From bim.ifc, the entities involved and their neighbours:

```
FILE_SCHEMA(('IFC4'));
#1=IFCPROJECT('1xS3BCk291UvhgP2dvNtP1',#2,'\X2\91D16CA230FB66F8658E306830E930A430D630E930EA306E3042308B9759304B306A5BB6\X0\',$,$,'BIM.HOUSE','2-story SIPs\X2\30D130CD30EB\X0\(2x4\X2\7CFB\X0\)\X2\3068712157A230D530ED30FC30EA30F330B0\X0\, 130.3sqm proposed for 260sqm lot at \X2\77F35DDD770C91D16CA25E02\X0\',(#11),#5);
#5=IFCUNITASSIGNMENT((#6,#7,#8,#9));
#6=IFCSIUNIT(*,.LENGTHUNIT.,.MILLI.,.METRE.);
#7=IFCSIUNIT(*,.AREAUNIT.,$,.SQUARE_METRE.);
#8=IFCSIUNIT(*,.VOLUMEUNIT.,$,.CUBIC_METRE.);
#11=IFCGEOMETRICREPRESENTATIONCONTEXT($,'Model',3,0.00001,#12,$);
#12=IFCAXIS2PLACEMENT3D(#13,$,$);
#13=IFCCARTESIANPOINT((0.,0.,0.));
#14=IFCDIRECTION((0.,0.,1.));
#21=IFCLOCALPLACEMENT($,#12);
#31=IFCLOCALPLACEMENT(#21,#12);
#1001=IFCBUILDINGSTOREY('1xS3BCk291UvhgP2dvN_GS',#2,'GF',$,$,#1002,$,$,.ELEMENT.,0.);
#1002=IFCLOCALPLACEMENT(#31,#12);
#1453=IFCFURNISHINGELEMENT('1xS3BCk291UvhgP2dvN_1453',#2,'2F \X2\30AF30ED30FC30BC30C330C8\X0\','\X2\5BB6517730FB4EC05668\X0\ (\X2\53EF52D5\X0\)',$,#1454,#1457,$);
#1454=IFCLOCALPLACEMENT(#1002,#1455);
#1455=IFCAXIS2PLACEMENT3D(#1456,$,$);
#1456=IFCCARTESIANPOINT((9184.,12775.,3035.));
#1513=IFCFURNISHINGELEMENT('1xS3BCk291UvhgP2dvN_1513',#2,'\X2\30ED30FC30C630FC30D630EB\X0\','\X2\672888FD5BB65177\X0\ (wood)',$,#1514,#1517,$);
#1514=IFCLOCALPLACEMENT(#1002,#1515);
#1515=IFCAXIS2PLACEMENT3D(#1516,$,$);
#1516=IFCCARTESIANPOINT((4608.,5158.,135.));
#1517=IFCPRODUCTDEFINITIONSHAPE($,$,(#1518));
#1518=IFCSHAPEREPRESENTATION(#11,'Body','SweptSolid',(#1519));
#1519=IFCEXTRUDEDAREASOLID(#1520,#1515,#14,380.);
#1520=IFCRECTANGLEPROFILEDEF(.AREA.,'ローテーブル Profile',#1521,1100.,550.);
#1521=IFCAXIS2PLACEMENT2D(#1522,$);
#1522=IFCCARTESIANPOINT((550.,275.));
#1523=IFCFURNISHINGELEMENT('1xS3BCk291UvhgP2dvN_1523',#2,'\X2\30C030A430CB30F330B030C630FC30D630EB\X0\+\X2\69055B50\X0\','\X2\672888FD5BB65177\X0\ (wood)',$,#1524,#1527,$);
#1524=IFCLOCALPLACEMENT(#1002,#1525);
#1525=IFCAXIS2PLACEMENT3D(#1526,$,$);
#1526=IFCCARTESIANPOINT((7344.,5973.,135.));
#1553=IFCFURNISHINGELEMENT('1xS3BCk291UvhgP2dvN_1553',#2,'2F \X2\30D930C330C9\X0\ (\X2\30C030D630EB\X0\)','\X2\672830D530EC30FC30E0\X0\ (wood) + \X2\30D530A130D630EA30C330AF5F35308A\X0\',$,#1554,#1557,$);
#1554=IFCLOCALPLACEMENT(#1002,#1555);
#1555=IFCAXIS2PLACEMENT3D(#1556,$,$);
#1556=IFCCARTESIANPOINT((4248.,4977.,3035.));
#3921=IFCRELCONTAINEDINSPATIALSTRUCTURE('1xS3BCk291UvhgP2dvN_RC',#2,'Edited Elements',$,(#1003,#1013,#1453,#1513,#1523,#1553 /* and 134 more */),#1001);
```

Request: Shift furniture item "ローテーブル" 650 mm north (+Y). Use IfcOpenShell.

```python
import ifcopenshell
import ifcopenshell.api.geometry
import ifcopenshell.util.placement
import ifcopenshell.util.unit

model = ifcopenshell.open("bim.ifc")
unit_scale = ifcopenshell.util.unit.calculate_unit_scale(model)

item = model.by_guid("1xS3BCk291UvhgP2dvN_1513")
matrix = ifcopenshell.util.placement.get_local_placement(item.ObjectPlacement)
matrix[1, 3] += 0.65 / unit_scale
ifcopenshell.api.geometry.edit_object_placement(model, product=item, matrix=matrix, is_si=False)

print(ifcopenshell.util.placement.get_local_placement(item.ObjectPlacement).round(3) + 0.0)

model.write("bim-out.ifc")
```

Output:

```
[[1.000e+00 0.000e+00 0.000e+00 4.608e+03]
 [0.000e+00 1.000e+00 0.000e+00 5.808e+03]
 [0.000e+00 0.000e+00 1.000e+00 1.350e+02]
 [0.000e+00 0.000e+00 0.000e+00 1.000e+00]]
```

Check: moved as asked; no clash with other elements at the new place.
